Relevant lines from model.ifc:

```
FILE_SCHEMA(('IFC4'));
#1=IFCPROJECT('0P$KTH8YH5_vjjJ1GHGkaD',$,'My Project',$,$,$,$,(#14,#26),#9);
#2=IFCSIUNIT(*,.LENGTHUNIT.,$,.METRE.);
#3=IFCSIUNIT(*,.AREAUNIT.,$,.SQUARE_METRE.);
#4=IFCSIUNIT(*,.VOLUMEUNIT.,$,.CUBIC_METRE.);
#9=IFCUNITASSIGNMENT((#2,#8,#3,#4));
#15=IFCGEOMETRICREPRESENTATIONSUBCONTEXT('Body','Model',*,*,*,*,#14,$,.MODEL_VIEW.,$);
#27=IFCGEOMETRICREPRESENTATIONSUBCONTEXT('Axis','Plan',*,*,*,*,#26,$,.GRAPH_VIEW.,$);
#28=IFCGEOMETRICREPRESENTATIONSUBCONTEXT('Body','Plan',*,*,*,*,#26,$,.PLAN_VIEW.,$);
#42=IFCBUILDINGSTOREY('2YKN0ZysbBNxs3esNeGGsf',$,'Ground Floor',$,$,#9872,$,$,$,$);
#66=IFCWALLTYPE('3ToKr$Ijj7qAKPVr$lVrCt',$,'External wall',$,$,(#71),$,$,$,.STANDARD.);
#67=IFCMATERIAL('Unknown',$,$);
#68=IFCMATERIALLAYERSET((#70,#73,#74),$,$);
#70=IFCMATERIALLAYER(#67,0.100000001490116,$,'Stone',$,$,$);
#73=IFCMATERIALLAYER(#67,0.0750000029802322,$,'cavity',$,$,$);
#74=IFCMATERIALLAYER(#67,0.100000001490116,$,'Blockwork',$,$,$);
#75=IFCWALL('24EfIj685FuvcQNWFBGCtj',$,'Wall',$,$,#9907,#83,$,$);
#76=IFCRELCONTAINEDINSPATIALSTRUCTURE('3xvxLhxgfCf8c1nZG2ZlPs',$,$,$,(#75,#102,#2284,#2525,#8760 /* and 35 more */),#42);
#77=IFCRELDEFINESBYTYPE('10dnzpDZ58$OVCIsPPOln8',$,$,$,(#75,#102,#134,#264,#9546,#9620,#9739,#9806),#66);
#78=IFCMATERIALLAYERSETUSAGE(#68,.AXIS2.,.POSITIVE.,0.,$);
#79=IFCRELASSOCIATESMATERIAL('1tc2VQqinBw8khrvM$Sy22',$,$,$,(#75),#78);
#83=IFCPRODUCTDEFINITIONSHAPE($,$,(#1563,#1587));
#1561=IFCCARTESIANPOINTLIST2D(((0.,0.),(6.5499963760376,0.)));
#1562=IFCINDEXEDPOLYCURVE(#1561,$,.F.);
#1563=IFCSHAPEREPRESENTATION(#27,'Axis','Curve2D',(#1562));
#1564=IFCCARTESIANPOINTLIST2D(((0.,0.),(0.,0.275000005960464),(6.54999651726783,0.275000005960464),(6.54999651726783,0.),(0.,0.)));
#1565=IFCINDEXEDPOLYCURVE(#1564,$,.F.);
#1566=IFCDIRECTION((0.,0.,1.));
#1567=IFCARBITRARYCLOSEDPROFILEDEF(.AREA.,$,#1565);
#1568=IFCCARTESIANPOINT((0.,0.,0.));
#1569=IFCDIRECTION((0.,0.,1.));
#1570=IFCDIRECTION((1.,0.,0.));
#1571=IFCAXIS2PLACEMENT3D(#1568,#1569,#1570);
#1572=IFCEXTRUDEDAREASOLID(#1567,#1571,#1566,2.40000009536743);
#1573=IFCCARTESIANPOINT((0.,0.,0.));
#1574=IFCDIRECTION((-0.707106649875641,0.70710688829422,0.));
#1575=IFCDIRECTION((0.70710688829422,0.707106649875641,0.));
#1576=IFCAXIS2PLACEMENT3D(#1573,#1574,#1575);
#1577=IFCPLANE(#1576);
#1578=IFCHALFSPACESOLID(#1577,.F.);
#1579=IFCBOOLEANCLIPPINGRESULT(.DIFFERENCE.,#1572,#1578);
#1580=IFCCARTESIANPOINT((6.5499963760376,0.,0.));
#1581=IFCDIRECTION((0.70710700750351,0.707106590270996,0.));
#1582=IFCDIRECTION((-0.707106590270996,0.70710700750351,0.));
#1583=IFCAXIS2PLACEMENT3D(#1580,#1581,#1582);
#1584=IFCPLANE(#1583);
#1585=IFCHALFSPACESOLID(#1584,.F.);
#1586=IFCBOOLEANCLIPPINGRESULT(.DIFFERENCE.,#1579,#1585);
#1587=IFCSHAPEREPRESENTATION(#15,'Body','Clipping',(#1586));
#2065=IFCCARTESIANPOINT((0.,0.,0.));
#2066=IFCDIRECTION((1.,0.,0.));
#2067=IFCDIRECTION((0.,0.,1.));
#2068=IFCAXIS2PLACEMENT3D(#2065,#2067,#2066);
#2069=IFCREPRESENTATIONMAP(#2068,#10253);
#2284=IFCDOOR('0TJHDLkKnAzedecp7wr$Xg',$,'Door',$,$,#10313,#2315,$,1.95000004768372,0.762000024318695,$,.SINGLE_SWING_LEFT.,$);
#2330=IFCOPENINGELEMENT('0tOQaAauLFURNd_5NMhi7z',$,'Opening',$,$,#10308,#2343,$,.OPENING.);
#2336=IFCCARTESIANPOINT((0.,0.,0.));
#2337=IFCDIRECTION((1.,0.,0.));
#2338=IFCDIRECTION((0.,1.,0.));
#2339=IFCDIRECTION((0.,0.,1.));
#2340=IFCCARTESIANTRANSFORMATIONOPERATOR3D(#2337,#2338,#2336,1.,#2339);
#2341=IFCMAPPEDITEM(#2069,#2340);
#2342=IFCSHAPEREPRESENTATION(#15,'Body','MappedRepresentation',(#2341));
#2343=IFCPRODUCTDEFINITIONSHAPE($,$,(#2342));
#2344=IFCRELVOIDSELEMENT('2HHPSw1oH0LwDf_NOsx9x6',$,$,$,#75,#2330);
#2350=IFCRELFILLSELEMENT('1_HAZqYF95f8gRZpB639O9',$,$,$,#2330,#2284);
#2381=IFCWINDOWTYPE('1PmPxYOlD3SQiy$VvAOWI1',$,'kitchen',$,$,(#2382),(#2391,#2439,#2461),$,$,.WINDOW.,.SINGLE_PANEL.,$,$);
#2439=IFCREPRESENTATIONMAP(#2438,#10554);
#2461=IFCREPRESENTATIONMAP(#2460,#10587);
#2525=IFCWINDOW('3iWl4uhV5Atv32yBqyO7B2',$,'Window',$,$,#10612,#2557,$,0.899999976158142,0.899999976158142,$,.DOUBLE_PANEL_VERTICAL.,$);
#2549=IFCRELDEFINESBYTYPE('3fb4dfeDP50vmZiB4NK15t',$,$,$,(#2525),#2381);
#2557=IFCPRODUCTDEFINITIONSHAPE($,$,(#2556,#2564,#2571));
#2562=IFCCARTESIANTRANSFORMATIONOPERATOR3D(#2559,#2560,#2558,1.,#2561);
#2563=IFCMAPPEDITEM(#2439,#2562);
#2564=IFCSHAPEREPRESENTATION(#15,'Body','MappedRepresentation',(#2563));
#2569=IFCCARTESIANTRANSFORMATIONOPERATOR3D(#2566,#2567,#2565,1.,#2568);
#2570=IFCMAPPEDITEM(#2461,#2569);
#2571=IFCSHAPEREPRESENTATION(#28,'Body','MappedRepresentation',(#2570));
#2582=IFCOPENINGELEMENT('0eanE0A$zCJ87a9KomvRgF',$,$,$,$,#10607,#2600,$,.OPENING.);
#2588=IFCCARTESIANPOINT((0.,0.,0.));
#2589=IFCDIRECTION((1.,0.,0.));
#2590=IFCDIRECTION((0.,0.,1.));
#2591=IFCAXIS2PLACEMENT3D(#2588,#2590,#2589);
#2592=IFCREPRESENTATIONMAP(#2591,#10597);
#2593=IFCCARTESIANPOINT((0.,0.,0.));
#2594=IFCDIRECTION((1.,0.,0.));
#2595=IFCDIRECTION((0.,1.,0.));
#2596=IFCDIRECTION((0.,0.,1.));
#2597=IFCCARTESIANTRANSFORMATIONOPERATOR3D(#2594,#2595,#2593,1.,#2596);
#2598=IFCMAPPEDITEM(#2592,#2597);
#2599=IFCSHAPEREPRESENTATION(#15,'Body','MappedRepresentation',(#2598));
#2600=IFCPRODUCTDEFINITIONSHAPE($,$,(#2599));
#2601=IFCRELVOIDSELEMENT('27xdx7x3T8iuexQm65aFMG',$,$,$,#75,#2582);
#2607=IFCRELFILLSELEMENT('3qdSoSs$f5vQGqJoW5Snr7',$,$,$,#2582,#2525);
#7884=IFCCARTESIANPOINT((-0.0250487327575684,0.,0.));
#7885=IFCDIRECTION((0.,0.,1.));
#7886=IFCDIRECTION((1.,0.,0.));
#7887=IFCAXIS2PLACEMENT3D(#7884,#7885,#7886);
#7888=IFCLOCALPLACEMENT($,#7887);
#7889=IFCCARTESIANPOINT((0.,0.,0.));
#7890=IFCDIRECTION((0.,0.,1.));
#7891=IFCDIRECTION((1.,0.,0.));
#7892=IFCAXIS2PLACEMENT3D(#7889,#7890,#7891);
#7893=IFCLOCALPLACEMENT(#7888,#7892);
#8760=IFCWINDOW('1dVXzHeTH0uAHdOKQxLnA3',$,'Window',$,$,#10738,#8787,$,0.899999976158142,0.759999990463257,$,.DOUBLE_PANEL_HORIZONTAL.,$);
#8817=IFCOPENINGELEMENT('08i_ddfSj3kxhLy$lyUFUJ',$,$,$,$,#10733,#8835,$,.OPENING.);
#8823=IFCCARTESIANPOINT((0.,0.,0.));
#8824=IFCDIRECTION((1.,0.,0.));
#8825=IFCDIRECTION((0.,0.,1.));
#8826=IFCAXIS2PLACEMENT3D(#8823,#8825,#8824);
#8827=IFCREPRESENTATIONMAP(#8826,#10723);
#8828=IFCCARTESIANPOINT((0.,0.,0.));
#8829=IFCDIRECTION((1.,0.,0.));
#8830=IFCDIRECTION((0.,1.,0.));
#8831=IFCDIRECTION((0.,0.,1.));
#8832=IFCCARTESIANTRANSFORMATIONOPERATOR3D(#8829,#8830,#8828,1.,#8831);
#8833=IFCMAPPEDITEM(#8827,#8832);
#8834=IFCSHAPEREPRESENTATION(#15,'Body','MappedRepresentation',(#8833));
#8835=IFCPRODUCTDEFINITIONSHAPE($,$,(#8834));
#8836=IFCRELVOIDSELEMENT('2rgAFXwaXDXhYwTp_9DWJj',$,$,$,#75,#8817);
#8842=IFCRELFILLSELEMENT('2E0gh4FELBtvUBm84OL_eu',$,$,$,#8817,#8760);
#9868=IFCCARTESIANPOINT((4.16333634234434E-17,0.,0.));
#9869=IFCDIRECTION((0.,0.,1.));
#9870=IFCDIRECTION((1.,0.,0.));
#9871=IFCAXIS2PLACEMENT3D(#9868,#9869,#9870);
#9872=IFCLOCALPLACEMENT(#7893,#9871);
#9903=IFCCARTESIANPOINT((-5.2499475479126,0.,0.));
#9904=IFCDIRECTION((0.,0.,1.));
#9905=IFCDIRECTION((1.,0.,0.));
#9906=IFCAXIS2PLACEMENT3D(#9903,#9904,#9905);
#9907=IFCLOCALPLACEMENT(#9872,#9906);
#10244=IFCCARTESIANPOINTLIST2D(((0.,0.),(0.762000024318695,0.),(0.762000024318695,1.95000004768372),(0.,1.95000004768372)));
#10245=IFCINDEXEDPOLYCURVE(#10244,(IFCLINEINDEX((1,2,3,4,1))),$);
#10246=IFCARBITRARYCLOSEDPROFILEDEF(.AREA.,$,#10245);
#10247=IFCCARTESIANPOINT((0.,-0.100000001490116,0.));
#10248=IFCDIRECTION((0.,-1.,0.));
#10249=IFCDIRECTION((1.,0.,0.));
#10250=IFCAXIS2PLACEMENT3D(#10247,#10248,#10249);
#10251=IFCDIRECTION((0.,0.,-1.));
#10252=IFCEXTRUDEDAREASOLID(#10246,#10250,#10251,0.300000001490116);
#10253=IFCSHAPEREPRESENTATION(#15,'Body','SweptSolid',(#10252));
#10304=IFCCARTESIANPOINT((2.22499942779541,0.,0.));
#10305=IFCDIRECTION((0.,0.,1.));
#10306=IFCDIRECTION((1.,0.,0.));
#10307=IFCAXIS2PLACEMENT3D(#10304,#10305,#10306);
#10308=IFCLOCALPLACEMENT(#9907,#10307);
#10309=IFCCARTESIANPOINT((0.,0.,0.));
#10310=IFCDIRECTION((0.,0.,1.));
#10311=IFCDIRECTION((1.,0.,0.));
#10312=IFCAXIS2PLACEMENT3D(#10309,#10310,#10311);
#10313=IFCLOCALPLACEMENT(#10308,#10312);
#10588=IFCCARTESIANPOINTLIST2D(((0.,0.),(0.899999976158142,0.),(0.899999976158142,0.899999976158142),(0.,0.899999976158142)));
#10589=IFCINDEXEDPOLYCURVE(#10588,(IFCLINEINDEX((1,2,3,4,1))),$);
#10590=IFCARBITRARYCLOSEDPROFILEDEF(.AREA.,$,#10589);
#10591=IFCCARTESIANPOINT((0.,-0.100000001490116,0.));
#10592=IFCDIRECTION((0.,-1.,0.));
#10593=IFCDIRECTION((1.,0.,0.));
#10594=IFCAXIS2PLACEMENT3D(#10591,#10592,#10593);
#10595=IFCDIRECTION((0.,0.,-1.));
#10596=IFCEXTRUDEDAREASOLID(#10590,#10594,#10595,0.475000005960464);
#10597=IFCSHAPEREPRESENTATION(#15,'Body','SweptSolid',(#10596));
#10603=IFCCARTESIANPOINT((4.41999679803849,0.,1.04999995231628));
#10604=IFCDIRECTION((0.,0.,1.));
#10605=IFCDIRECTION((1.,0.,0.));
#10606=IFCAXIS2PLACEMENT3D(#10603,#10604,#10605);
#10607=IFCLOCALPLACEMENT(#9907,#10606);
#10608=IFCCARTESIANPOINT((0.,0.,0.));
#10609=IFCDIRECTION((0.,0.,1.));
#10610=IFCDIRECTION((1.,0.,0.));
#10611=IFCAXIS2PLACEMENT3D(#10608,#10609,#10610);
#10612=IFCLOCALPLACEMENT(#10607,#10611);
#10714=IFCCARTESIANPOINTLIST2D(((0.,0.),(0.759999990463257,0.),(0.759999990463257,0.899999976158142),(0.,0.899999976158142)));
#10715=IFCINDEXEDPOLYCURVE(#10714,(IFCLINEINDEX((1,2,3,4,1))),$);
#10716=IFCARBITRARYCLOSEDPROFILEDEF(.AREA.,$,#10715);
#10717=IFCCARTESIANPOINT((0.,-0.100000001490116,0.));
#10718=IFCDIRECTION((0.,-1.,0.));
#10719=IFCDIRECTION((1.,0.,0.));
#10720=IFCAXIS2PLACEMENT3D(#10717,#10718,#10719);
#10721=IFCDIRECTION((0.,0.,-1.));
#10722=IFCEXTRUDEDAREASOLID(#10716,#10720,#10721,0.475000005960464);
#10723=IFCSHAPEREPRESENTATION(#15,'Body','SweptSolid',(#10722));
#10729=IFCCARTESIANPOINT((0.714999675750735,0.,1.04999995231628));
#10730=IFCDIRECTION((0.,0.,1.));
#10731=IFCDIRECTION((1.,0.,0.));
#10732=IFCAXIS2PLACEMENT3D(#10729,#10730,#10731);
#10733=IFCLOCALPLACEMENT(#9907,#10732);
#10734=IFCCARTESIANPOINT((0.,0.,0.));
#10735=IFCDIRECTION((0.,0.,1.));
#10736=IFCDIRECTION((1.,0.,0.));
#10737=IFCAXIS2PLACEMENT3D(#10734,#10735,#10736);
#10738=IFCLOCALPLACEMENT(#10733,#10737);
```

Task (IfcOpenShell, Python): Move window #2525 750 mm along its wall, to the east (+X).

```python
import ifcopenshell
import ifcopenshell.api.geometry
import ifcopenshell.util.placement
import ifcopenshell.util.unit

model = ifcopenshell.open("model.ifc")
unit_scale = ifcopenshell.util.unit.calculate_unit_scale(model)

window = model.by_id(2525)
opening = window.FillsVoids[0].RelatingOpeningElement
wall = opening.VoidsElements[0].RelatingBuildingElement

wall_matrix = ifcopenshell.util.placement.get_local_placement(wall.ObjectPlacement)
shift = wall_matrix[:3, 0] * 0.75 / unit_scale
before = ifcopenshell.util.placement.get_local_placement(window.ObjectPlacement)[:3, 3].copy()

# The window is placed relative to its opening, so it follows when the opening moves.
matrix = ifcopenshell.util.placement.get_local_placement(opening.ObjectPlacement)
matrix[:3, 3] += shift
ifcopenshell.api.geometry.edit_object_placement(
    model, product=opening, matrix=matrix, is_si=False, should_transform_children=True
)

after = ifcopenshell.util.placement.get_local_placement(window.ObjectPlacement)[:3, 3]
print("window moved by", (after - before).round(3) + 0.0)

model.write("model_edited.ifc")
```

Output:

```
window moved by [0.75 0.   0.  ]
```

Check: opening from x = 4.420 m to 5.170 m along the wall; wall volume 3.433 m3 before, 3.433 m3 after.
